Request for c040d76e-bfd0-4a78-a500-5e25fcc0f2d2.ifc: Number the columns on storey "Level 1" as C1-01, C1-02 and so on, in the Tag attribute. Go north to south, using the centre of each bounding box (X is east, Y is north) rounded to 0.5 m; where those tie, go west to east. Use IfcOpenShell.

First a look at what the model holds.

```python
import ifcopenshell
import ifcopenshell.util.element
import ifcopenshell.util.placement

model = ifcopenshell.open("c040d76e-bfd0-4a78-a500-5e25fcc0f2d2.ifc")
print(model.schema)
storey = next(s for s in model.by_type("IfcBuildingStorey") if s.Name == "Level 1")
columns = [e for e in ifcopenshell.util.element.get_decomposition(storey) if e.is_a("IfcColumn")]
for e in sorted(columns, key=lambda e: e.id()):
    origin = ifcopenshell.util.placement.get_local_placement(e.ObjectPlacement)[:3, 3]
    print(e.id(), e.Tag, e.Name, origin.round(2) + 0.0, sep=" | ")
```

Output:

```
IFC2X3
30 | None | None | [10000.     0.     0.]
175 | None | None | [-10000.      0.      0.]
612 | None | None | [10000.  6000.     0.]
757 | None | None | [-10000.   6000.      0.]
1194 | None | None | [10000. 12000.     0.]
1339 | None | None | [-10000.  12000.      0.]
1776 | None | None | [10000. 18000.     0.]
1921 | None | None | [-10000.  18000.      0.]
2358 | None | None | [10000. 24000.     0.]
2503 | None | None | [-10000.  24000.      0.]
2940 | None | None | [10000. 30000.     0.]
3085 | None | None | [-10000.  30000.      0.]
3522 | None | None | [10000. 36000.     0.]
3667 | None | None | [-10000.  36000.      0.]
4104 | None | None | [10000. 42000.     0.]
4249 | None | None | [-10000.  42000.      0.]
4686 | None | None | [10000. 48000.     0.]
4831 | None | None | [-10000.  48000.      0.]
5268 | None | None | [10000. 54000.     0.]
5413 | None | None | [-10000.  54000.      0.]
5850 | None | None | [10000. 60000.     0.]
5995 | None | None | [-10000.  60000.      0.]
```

```python
import ifcopenshell
import ifcopenshell.geom
import ifcopenshell.util.element
import ifcopenshell.util.shape

model = ifcopenshell.open("c040d76e-bfd0-4a78-a500-5e25fcc0f2d2.ifc")
settings = ifcopenshell.geom.settings()
settings.set("use-world-coords", True)


def centre(element):
    shape = ifcopenshell.geom.create_shape(settings, element)
    return ifcopenshell.util.shape.get_bbox_centroid(shape.geometry)


storey = next(s for s in model.by_type("IfcBuildingStorey") if s.Name == "Level 1")
columns = [e for e in ifcopenshell.util.element.get_decomposition(storey) if e.is_a("IfcColumn")]

# Insertion points can sit at a corner or the storey origin, so sort by the geometry (in metres).
centres = {e: centre(e) for e in columns}
columns.sort(key=lambda e: (-round(centres[e][1] / 0.5), centres[e][0]))

for i, e in enumerate(columns, start=1):
    number = f"C1-{i:02d}"
    e.Tag = number
    print(e.id(), number)

model.write("c040d76e-bfd0-4a78-a500-5e25fcc0f2d2_edited.ifc")
```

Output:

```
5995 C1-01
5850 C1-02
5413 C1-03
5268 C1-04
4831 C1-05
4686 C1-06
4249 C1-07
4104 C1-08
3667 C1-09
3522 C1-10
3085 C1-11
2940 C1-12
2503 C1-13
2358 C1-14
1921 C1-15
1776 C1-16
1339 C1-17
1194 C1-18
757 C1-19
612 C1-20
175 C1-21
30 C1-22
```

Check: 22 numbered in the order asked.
